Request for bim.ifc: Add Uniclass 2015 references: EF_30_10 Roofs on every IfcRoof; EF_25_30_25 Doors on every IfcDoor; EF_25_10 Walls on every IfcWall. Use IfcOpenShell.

First a look at what the model holds.

```python
import ifcopenshell

model = ifcopenshell.open("bim.ifc")
print(model.schema)
print("classifications:", [c.Name for c in model.by_type("IfcClassification")])
for ifc_class in ("IfcDoor", "IfcRoof", "IfcStair", "IfcWall", "IfcWindow"):
    print(ifc_class, len(model.by_type(ifc_class)))
```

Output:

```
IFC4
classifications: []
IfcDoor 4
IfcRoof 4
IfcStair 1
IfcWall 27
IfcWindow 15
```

```python
import ifcopenshell
import ifcopenshell.api.classification

model = ifcopenshell.open("bim.ifc")

system = ifcopenshell.api.classification.add_classification(model, classification="Uniclass 2015")

codes = {
    "IfcRoof": ("EF_30_10", "Roofs"),
    "IfcDoor": ("EF_25_30_25", "Doors"),
    "IfcWall": ("EF_25_10", "Walls"),
}
for ifc_class, (code, name) in codes.items():
    products = model.by_type(ifc_class)
    ifcopenshell.api.classification.add_reference(
        model, products=products, classification=system, identification=code, name=name
    )
    print(code, len(products))

model.write("bim_rev.ifc")
```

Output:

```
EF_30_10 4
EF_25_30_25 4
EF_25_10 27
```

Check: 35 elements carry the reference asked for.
